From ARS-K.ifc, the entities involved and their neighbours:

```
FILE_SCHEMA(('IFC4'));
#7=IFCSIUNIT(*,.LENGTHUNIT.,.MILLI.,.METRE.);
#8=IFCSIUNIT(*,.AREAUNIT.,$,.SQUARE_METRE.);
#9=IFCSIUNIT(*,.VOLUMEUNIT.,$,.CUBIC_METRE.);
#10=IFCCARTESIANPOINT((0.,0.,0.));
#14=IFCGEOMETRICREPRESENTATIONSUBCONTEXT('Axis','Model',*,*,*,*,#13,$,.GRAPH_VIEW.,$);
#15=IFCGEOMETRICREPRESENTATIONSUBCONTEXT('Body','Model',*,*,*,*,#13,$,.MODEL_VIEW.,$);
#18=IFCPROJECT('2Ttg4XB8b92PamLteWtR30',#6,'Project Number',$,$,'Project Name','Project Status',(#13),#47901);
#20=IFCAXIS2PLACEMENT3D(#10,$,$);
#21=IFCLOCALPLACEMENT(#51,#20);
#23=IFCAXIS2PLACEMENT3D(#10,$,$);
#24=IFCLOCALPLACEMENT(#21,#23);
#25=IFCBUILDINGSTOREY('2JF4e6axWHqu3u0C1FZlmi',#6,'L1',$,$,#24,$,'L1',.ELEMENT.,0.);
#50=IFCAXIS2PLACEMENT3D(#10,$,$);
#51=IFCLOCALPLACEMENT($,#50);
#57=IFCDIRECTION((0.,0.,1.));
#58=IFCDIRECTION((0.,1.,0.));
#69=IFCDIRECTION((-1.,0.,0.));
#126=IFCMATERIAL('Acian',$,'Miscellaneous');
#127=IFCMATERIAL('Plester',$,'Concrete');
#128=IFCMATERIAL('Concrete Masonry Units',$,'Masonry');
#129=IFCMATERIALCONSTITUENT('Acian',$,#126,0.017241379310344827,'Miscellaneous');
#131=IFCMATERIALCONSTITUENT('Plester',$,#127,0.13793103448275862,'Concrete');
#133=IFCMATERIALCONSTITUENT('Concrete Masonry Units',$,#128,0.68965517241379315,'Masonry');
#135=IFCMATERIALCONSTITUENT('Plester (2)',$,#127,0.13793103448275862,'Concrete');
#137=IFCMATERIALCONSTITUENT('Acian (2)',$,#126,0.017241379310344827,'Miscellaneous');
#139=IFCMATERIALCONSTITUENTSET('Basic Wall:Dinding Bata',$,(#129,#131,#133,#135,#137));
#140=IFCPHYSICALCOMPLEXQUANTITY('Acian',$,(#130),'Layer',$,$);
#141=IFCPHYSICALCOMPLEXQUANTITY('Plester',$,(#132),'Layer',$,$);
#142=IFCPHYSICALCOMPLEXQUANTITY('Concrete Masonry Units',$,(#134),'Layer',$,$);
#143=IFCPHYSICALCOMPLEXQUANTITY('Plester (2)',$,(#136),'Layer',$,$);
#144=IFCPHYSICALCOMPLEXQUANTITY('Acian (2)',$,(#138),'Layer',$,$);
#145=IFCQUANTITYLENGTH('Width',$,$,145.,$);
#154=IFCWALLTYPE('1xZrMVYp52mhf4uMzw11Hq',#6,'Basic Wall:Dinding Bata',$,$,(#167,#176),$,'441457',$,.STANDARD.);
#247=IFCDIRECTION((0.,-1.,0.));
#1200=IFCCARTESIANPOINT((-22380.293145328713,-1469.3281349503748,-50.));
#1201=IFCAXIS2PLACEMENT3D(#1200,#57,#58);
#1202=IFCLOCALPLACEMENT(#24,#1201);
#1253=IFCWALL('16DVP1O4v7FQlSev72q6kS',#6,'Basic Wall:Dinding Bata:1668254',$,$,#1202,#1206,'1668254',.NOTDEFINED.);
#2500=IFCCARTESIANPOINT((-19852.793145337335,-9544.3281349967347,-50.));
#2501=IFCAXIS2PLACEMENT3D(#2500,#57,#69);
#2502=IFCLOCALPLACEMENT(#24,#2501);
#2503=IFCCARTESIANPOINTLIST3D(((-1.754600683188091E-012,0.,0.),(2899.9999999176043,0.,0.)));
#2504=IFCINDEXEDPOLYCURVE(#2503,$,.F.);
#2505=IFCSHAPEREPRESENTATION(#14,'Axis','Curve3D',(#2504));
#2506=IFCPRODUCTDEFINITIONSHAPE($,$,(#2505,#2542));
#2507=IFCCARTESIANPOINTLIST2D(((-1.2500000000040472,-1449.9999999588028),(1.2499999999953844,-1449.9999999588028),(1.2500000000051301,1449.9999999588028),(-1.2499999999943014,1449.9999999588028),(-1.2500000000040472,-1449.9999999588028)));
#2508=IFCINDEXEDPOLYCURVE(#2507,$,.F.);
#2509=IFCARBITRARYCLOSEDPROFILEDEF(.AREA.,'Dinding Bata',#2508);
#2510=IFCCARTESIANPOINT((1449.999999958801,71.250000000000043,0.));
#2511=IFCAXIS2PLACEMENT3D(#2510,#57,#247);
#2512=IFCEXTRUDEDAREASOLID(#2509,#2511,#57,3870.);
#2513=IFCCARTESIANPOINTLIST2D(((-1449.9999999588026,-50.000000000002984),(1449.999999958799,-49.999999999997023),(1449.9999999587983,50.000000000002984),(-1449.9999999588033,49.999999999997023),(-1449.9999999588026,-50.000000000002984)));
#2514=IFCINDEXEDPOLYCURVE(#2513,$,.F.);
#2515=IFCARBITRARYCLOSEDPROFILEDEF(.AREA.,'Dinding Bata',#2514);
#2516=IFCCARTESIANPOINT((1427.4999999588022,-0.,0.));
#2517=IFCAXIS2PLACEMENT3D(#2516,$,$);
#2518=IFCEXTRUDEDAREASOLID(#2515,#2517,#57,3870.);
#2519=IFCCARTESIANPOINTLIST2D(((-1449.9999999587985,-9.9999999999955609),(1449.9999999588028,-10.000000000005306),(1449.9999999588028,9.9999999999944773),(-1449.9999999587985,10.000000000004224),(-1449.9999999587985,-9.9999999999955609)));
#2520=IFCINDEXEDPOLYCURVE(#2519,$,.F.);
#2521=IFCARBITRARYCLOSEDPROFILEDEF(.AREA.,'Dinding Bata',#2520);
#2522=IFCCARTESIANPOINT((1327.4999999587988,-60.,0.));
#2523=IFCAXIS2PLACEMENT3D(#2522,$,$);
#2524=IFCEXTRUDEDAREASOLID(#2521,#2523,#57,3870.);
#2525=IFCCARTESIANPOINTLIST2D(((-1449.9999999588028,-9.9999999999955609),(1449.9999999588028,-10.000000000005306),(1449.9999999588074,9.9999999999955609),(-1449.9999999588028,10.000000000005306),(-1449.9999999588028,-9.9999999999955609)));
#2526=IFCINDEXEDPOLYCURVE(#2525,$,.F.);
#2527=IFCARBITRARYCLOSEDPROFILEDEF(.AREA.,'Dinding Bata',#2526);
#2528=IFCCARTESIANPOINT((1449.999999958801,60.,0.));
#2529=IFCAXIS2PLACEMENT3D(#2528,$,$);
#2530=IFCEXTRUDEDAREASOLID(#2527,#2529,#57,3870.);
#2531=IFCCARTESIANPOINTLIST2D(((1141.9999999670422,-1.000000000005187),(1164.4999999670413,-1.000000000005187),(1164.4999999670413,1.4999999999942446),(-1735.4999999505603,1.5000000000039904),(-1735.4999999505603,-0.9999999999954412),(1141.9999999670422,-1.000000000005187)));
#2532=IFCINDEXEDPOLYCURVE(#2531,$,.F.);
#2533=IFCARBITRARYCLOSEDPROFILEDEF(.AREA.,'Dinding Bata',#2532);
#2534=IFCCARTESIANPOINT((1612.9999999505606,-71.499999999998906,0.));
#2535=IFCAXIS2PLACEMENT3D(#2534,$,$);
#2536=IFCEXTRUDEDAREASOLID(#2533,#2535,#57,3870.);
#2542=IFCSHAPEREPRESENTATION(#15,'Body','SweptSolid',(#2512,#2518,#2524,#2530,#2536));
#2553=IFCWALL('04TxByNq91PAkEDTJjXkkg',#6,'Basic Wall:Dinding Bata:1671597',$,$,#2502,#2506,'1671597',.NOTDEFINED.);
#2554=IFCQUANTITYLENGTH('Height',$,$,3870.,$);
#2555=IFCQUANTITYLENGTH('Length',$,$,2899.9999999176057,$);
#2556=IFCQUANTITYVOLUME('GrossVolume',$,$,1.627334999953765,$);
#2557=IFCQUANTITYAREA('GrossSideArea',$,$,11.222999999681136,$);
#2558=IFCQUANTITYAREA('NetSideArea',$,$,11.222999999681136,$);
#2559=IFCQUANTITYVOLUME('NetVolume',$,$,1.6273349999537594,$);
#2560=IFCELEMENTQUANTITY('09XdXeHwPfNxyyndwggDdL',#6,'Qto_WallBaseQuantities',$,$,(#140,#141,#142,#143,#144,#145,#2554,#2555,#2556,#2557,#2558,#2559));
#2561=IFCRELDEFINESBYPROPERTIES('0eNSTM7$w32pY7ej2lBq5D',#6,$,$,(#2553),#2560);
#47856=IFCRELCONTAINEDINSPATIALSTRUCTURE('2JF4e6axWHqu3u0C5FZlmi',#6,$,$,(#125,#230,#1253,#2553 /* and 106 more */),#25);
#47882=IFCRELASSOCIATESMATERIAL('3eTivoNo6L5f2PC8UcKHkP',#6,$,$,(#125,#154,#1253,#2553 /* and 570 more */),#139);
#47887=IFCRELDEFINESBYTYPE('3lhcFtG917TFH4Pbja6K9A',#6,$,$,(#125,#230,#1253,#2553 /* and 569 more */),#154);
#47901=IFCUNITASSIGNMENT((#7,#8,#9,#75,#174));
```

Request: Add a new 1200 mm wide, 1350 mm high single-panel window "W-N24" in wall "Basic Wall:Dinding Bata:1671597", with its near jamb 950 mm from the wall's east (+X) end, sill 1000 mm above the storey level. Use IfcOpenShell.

```python
import numpy as np
import ifcopenshell
import ifcopenshell.api.feature
import ifcopenshell.api.geometry
import ifcopenshell.api.pset
import ifcopenshell.api.root
import ifcopenshell.api.spatial
import ifcopenshell.geom
import ifcopenshell.util.element
import ifcopenshell.util.placement
import ifcopenshell.util.representation
import ifcopenshell.util.shape
import ifcopenshell.util.unit

model = ifcopenshell.open("ARS-K.ifc")
unit_scale = ifcopenshell.util.unit.calculate_unit_scale(model)
area_scale = ifcopenshell.util.unit.calculate_unit_scale(model, "AREAUNIT")
volume_scale = ifcopenshell.util.unit.calculate_unit_scale(model, "VOLUMEUNIT")
settings = ifcopenshell.geom.settings()


def volume(element):
    """Net volume in cubic metres, openings subtracted."""
    shape = ifcopenshell.geom.create_shape(settings, element)
    return ifcopenshell.util.shape.get_volume(shape.geometry)


wall = model.by_id(2553)
storey = ifcopenshell.util.element.get_container(wall, ifc_class="IfcBuildingStorey")
context = ifcopenshell.util.representation.get_context(model, "Model", "Body", "MODEL_VIEW")
before = volume(wall)

width, height, from_end, sill = 1.2, 1.35, 0.95, 1  # metres

# The wall runs along its own X axis, and the end named is its -X end.
wall_shape = ifcopenshell.geom.create_shape(settings, wall)
x, y, z = ifcopenshell.util.shape.get_vertices(wall_shape.geometry).T
start = x.min() + from_end
face, thickness = float(y.min()), float(y.max() - y.min())
wall_matrix = ifcopenshell.util.placement.get_local_placement(wall.ObjectPlacement)
level = ifcopenshell.util.placement.get_local_placement(storey.ObjectPlacement)[2, 3]


def in_wall(x, y):
    """Placement at x, y metres in the wall's axes, at sill height."""
    matrix = wall_matrix.copy()
    matrix[:, 3] = wall_matrix @ np.array([x / unit_scale, y / unit_scale, 0.0, 1.0])
    matrix[2, 3] = level + sill / unit_scale
    return matrix


# Opening: a box that overshoots both wall faces by 50 mm.
opening = ifcopenshell.api.root.create_entity(model, ifc_class="IfcOpeningElement", predefined_type="OPENING")
box = ifcopenshell.api.geometry.add_wall_representation(
    model, context=context, length=width, height=height, thickness=thickness + 0.1
)
ifcopenshell.api.geometry.assign_representation(model, product=opening, representation=box)
ifcopenshell.api.geometry.edit_object_placement(model, product=opening, matrix=in_wall(start, face - 0.05), is_si=False)
ifcopenshell.api.feature.add_feature(model, feature=opening, element=wall)

window = ifcopenshell.api.root.create_entity(model, ifc_class="IfcWindow", name="W-N24", predefined_type="WINDOW")
window.OverallWidth, window.OverallHeight = width / unit_scale, height / unit_scale
window.PartitioningType = "SINGLE_PANEL"
body = ifcopenshell.api.geometry.add_window_representation(
    model,
    context=context,
    overall_width=window.OverallWidth,
    overall_height=window.OverallHeight,
    partition_type="SINGLE_PANEL",
)
ifcopenshell.api.geometry.assign_representation(model, product=window, representation=body)
ifcopenshell.api.spatial.assign_container(model, products=[window], relating_structure=storey)
ifcopenshell.api.feature.add_filling(model, opening=opening, element=window)

# Centre the window in the wall's thickness.
ifcopenshell.api.geometry.edit_object_placement(model, product=window, matrix=in_wall(start, face), is_si=False)
window_shape = ifcopenshell.geom.create_shape(settings, window)
depth = ifcopenshell.util.shape.get_vertices(window_shape.geometry)[:, 1]
offset = face + thickness / 2 - (depth.min() + depth.max()) / 2
ifcopenshell.api.geometry.edit_object_placement(model, product=window, matrix=in_wall(start, offset), is_si=False)

after = volume(wall)

# Update the wall's stored quantities.
qto = model.by_id(ifcopenshell.util.element.get_pset(wall, "Qto_WallBaseQuantities", should_inherit=False)["id"])
ifcopenshell.api.pset.edit_qto(model, qto=qto, properties={
    "NetSideArea": after / thickness / area_scale,
    "NetVolume": after / volume_scale,
})

print(f"wall volume {before:.3f} -> {after:.3f} m3")

model.write("ARS-K_updated.ifc")
```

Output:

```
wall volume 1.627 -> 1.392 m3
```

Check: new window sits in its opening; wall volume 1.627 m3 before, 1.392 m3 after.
